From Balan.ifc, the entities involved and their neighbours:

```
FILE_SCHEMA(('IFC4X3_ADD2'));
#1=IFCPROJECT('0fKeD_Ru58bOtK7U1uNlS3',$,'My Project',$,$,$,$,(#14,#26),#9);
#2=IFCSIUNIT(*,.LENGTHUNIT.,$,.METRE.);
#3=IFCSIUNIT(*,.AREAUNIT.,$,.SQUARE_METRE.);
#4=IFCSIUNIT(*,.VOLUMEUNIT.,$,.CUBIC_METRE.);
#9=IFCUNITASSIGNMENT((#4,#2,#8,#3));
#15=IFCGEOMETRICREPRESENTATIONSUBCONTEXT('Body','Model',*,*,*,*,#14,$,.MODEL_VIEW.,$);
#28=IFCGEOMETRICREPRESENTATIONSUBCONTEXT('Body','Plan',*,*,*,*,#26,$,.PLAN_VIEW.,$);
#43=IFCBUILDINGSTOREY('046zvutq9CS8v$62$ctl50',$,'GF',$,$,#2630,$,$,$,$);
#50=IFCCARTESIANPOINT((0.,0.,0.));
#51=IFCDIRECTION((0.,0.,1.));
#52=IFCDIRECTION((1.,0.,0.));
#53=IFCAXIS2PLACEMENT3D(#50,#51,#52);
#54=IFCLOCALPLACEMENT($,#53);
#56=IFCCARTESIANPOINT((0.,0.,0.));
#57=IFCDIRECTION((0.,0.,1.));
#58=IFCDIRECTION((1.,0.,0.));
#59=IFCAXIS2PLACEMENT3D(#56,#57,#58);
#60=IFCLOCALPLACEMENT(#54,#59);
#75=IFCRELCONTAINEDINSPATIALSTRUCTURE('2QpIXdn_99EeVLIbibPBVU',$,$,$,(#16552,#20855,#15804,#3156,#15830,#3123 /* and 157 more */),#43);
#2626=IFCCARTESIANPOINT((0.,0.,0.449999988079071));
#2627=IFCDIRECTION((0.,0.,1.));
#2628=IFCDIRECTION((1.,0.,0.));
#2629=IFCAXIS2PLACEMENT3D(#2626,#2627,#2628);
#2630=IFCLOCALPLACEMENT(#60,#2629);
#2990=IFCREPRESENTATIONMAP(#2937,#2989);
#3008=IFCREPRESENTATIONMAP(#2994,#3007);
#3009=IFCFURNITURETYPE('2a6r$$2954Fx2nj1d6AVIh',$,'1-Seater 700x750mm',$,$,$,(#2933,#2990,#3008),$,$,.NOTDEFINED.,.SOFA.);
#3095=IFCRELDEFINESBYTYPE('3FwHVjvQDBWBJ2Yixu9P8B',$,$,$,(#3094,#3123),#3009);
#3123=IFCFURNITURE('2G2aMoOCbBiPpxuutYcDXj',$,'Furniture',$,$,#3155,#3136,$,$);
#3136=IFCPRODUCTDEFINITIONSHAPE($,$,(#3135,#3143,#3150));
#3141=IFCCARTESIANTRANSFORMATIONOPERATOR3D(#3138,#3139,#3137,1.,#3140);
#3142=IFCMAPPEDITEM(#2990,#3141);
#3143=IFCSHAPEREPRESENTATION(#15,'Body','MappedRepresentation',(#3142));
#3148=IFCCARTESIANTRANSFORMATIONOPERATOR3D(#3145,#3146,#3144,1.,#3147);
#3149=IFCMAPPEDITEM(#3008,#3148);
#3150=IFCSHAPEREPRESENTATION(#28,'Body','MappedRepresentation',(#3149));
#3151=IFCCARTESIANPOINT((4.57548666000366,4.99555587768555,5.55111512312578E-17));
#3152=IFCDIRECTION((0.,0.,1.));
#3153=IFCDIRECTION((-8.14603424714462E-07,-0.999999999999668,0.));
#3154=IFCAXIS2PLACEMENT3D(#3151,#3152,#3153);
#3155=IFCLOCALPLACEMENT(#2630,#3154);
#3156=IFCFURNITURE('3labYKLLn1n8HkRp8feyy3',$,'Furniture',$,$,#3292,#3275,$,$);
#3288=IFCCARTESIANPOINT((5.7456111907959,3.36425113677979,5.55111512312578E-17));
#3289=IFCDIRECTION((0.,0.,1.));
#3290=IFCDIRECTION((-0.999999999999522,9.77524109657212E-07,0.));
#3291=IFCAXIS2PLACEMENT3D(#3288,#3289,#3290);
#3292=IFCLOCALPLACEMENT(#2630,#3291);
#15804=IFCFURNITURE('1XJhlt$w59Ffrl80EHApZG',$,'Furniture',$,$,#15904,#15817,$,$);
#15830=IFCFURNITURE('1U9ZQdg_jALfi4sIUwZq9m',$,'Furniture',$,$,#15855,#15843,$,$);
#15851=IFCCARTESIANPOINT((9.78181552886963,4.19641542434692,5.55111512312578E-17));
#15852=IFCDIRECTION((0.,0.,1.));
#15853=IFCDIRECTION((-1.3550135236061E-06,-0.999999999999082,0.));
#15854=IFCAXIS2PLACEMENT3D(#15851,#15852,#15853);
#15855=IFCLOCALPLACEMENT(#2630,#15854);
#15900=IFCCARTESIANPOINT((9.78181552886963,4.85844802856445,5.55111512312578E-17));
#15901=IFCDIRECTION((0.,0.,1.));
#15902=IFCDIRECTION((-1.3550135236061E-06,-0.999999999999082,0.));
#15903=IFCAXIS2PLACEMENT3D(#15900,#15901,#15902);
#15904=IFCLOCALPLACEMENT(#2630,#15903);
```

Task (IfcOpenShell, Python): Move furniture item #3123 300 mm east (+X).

```python
import ifcopenshell
import ifcopenshell.api.geometry
import ifcopenshell.util.placement
import ifcopenshell.util.unit

model = ifcopenshell.open("Balan.ifc")
unit_scale = ifcopenshell.util.unit.calculate_unit_scale(model)

item = model.by_guid("2G2aMoOCbBiPpxuutYcDXj")
matrix = ifcopenshell.util.placement.get_local_placement(item.ObjectPlacement)
matrix[0, 3] += 0.3 / unit_scale
ifcopenshell.api.geometry.edit_object_placement(model, product=item, matrix=matrix, is_si=False)

print(ifcopenshell.util.placement.get_local_placement(item.ObjectPlacement).round(3) + 0.0)

model.write("Balan_updated.ifc")
```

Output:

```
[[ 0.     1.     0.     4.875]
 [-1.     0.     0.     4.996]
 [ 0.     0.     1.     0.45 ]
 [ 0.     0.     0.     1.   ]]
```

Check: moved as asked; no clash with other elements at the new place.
